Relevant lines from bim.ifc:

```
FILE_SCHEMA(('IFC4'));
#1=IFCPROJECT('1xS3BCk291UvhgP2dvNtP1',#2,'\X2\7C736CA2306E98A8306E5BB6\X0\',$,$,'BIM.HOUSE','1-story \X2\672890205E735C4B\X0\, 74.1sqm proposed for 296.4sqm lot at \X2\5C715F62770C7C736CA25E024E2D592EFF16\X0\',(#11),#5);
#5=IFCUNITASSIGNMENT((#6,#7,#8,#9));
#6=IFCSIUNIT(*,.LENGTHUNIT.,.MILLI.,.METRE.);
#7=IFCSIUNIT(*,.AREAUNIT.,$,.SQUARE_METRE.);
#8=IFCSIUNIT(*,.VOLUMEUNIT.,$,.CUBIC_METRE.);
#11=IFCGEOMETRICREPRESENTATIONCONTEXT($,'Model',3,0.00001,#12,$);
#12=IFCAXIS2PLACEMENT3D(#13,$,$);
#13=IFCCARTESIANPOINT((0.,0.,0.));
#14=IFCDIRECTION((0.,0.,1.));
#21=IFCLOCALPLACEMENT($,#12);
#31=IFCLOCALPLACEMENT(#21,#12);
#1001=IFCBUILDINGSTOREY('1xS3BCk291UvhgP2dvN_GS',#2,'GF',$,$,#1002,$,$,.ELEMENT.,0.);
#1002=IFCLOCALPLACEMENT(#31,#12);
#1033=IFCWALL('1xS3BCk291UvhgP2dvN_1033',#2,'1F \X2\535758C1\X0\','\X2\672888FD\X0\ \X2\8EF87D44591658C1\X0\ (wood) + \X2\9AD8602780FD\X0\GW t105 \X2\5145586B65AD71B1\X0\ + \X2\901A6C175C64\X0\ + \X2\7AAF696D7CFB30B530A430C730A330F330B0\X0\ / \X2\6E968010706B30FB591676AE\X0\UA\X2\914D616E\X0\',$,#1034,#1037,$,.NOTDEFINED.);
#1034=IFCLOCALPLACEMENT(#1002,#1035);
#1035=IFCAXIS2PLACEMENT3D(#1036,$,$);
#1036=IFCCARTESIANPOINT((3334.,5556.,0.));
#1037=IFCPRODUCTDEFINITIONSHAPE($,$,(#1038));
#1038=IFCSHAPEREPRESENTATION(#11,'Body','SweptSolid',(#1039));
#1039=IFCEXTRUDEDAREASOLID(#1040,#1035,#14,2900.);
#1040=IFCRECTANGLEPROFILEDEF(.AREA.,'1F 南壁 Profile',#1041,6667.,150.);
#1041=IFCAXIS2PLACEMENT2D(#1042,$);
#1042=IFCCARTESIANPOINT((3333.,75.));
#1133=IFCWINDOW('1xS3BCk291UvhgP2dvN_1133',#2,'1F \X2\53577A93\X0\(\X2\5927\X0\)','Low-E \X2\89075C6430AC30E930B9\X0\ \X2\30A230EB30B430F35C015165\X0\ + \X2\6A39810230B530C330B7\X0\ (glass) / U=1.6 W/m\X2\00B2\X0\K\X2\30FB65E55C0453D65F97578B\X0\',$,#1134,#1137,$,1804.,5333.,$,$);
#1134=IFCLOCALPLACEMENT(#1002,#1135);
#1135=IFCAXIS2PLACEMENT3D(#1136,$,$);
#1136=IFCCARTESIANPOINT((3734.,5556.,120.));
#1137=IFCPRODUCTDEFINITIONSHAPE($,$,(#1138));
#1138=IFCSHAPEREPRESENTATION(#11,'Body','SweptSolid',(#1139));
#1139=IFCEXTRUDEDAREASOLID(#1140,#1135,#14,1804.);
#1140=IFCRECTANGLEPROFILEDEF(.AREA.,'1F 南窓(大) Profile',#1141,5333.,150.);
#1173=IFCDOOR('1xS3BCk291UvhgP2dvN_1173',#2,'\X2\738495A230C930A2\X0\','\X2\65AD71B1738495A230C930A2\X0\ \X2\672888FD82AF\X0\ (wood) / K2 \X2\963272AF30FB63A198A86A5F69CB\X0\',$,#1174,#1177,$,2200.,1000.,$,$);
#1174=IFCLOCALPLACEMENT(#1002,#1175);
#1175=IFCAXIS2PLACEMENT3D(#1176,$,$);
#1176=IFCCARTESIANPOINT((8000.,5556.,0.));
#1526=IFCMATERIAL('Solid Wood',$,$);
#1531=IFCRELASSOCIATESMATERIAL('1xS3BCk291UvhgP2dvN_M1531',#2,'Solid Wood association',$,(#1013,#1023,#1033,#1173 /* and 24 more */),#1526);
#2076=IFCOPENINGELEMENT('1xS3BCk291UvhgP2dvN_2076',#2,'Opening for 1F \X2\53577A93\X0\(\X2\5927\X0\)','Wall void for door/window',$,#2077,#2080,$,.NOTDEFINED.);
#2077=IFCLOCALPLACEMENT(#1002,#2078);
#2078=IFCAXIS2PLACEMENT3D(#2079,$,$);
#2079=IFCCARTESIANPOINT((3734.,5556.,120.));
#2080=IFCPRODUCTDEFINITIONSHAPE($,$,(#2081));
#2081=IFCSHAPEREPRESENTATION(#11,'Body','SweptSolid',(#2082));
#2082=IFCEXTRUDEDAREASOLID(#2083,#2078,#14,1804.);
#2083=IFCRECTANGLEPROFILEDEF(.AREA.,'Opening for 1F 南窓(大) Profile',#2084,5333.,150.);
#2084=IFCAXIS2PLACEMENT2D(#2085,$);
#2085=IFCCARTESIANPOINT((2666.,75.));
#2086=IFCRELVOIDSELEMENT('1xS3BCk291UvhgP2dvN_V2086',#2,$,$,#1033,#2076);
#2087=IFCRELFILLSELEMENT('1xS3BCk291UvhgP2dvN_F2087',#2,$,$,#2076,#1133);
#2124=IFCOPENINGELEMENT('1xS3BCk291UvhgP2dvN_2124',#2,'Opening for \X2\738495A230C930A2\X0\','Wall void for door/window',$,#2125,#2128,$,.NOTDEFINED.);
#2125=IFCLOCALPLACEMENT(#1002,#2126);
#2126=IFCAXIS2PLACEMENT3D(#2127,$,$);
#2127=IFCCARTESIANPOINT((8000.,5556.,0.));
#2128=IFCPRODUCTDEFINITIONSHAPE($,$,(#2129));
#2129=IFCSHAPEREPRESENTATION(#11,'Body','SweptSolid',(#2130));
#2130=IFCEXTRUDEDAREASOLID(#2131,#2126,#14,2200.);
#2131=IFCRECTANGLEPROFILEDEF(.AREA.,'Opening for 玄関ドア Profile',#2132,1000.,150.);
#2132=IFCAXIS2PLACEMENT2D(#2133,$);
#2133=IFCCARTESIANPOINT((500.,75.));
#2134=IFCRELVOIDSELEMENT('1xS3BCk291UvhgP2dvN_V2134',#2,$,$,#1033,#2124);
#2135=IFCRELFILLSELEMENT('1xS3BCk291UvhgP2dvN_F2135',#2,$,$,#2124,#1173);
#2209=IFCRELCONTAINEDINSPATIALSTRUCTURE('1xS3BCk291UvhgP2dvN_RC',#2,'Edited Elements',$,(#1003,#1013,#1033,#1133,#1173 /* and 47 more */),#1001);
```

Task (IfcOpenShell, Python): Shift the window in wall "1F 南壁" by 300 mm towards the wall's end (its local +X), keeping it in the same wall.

```python
import ifcopenshell
import ifcopenshell.api.geometry
import ifcopenshell.util.placement

model = ifcopenshell.open("bim.ifc")

window = model.by_id(1133)
opening = window.FillsVoids[0].RelatingOpeningElement
wall = opening.VoidsElements[0].RelatingBuildingElement

wall_matrix = ifcopenshell.util.placement.get_local_placement(wall.ObjectPlacement)
shift = wall_matrix[:3, 0] * 300.0
before = ifcopenshell.util.placement.get_local_placement(window.ObjectPlacement)[:3, 3].copy()

# The window is not placed relative to its opening, so move both.
for product in (opening, window):
    matrix = ifcopenshell.util.placement.get_local_placement(product.ObjectPlacement)
    matrix[:3, 3] += shift
    ifcopenshell.api.geometry.edit_object_placement(model, product=product, matrix=matrix, is_si=False)

after = ifcopenshell.util.placement.get_local_placement(window.ObjectPlacement)[:3, 3]
print("window moved by", (after - before).round(3) + 0.0)

model.write("bim_v2.ifc")
```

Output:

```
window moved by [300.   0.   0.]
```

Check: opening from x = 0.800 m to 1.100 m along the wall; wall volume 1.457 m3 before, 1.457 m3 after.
